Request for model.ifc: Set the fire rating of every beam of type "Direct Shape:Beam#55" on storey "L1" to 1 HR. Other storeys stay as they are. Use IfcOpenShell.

First a look at what the model holds.

```python
import ifcopenshell
import ifcopenshell.util.element

model = ifcopenshell.open("model.ifc")
print(model.schema)
storey = next(s for s in model.by_type("IfcBuildingStorey") if s.Name == "L1")
beams = [e for e in ifcopenshell.util.element.get_decomposition(storey) if e.is_a("IfcBeam")]
seen = {}
for e in beams:
    element_type = ifcopenshell.util.element.get_type(e)
    key = (element_type.Name if element_type != e and element_type else None, ifcopenshell.util.element.get_pset(e, "Pset_BeamCommon", "FireRating"))
    seen[key] = seen.get(key, 0) + 1
for (name, value), count in sorted(seen.items(), key=str):
    print(count, "x", name, "|", value)
```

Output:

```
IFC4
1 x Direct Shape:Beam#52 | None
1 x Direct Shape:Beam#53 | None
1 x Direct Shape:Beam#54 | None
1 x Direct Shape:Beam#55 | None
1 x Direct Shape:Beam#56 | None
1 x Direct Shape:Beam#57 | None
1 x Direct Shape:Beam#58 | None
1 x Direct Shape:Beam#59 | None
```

```python
import ifcopenshell
import ifcopenshell.api.pset
import ifcopenshell.util.element

model = ifcopenshell.open("model.ifc")

storey = next(s for s in model.by_type("IfcBuildingStorey") if s.Name == "L1")
beams = [e for e in ifcopenshell.util.element.get_decomposition(storey) if e.is_a("IfcBeam")]

count = 0
for e in beams:
    element_type = ifcopenshell.util.element.get_type(e)
    if element_type in (None, e) or element_type.Name != "Direct Shape:Beam#55":
        continue
    # add_pset returns the element's existing set when there is one.
    pset = ifcopenshell.api.pset.add_pset(model, product=e, name="Pset_BeamCommon")
    ifcopenshell.api.pset.edit_pset(model, pset=pset, properties={"FireRating": "1 HR"})
    count += 1

print(count, "beams updated")

model.write("model_edited.ifc")
```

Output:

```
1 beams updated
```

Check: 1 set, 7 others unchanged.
